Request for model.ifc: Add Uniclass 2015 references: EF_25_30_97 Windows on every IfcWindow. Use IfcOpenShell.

First a look at what the model holds.

```python
import ifcopenshell

model = ifcopenshell.open("model.ifc")
print(model.schema)
print("classifications:", [c.Name for c in model.by_type("IfcClassification")])
for ifc_class in ("IfcDoor", "IfcRoof", "IfcStair", "IfcWall", "IfcWindow"):
    print(ifc_class, len(model.by_type(ifc_class)))
```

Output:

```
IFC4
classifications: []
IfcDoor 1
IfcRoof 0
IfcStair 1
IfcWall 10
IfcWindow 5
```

```python
import ifcopenshell
import ifcopenshell.api.classification

model = ifcopenshell.open("model.ifc")

system = ifcopenshell.api.classification.add_classification(model, classification="Uniclass 2015")

codes = {
    "IfcWindow": ("EF_25_30_97", "Windows"),
}
for ifc_class, (code, name) in codes.items():
    products = model.by_type(ifc_class)
    ifcopenshell.api.classification.add_reference(
        model, products=products, classification=system, identification=code, name=name
    )
    print(code, len(products))

model.write("model_rev.ifc")
```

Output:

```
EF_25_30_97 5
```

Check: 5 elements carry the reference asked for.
